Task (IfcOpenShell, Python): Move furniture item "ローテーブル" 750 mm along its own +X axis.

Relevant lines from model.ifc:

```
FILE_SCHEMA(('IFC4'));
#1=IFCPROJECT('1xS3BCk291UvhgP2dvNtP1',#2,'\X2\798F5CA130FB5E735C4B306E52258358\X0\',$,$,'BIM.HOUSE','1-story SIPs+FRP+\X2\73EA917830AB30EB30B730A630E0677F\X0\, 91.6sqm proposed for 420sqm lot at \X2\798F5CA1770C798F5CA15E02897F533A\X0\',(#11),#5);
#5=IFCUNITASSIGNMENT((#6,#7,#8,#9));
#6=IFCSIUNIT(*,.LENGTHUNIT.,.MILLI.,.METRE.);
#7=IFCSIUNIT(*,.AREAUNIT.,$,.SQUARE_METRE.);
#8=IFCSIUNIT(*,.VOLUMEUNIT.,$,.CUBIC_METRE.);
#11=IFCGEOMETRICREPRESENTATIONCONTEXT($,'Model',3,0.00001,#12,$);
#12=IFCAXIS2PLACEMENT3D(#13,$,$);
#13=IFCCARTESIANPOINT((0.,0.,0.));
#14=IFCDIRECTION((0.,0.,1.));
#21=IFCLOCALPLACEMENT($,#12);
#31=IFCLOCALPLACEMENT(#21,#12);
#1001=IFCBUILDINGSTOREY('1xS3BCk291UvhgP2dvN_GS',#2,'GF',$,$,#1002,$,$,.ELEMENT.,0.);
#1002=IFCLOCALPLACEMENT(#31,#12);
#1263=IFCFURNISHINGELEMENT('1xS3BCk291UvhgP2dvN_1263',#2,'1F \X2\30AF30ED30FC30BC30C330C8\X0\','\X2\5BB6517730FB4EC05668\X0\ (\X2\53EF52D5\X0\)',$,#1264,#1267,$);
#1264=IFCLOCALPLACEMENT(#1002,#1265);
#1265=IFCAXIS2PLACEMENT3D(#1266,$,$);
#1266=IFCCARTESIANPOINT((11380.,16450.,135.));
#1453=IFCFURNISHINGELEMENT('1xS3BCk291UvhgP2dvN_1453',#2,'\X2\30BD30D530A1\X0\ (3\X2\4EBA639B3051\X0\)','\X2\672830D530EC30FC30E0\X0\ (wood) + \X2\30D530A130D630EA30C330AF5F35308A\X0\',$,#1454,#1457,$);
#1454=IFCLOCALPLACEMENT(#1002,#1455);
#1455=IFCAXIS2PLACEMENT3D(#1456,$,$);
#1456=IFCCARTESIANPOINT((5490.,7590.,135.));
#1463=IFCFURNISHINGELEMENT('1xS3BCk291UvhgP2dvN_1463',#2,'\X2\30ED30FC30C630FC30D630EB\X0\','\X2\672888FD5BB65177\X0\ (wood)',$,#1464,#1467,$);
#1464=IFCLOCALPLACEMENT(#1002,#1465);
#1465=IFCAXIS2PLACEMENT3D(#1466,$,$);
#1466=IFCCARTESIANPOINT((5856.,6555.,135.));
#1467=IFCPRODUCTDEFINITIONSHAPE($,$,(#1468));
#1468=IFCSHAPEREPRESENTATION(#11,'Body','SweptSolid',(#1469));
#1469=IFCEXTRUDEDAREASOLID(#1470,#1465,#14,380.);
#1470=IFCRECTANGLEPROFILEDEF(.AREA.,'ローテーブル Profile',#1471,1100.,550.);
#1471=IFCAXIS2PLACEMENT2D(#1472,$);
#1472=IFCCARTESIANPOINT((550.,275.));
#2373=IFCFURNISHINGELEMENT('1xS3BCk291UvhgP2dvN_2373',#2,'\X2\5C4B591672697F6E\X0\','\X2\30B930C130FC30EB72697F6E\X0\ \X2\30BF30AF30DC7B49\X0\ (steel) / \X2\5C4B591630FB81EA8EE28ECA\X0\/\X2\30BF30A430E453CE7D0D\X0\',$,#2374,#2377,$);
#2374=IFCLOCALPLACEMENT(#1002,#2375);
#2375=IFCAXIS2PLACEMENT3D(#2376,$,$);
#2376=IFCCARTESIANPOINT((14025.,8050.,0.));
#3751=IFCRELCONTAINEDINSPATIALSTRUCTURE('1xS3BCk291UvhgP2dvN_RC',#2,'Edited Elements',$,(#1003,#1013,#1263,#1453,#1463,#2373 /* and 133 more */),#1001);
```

```python
import ifcopenshell
import ifcopenshell.api.geometry
import ifcopenshell.util.placement

model = ifcopenshell.open("model.ifc")

item = model.by_guid("1xS3BCk291UvhgP2dvN_1463")
matrix = ifcopenshell.util.placement.get_local_placement(item.ObjectPlacement)
matrix[:3, 3] += matrix[:3, 0] * 750.0
ifcopenshell.api.geometry.edit_object_placement(model, product=item, matrix=matrix, is_si=False)

print(ifcopenshell.util.placement.get_local_placement(item.ObjectPlacement).round(3) + 0.0)

model.write("model-out.ifc")
```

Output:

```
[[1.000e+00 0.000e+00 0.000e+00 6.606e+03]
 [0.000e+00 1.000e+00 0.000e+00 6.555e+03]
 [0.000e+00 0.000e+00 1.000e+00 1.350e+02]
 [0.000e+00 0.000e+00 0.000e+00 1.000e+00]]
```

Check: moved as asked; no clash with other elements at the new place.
